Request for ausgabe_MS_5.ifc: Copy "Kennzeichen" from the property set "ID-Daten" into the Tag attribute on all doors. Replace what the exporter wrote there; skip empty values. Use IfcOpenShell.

First a look at what the model holds.

```python
import ifcopenshell
import ifcopenshell.util.element

model = ifcopenshell.open("ausgabe_MS_5.ifc")
print(model.schema)
doors = model.by_type("IfcDoor")
print(len(doors), "doors")
for e in doors[:8]:
    source = ifcopenshell.util.element.get_pset(e, "ID-Daten", "Kennzeichen")
    target = e.Tag
    print(e.id(), repr(source), repr(target), sep=" | ")
```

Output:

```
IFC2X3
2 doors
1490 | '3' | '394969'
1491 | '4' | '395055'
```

```python
import ifcopenshell
import ifcopenshell.util.element

model = ifcopenshell.open("ausgabe_MS_5.ifc")

count = 0
for e in model.by_type("IfcDoor"):
    value = ifcopenshell.util.element.get_pset(e, "ID-Daten", "Kennzeichen")
    current = e.Tag
    if not value or not value.strip() or current == value:
        continue
    e.Tag = value
    count += 1

print(count, "doors updated")

model.write("ausgabe_MS_5_v2.ifc")
```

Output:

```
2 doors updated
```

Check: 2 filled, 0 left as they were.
